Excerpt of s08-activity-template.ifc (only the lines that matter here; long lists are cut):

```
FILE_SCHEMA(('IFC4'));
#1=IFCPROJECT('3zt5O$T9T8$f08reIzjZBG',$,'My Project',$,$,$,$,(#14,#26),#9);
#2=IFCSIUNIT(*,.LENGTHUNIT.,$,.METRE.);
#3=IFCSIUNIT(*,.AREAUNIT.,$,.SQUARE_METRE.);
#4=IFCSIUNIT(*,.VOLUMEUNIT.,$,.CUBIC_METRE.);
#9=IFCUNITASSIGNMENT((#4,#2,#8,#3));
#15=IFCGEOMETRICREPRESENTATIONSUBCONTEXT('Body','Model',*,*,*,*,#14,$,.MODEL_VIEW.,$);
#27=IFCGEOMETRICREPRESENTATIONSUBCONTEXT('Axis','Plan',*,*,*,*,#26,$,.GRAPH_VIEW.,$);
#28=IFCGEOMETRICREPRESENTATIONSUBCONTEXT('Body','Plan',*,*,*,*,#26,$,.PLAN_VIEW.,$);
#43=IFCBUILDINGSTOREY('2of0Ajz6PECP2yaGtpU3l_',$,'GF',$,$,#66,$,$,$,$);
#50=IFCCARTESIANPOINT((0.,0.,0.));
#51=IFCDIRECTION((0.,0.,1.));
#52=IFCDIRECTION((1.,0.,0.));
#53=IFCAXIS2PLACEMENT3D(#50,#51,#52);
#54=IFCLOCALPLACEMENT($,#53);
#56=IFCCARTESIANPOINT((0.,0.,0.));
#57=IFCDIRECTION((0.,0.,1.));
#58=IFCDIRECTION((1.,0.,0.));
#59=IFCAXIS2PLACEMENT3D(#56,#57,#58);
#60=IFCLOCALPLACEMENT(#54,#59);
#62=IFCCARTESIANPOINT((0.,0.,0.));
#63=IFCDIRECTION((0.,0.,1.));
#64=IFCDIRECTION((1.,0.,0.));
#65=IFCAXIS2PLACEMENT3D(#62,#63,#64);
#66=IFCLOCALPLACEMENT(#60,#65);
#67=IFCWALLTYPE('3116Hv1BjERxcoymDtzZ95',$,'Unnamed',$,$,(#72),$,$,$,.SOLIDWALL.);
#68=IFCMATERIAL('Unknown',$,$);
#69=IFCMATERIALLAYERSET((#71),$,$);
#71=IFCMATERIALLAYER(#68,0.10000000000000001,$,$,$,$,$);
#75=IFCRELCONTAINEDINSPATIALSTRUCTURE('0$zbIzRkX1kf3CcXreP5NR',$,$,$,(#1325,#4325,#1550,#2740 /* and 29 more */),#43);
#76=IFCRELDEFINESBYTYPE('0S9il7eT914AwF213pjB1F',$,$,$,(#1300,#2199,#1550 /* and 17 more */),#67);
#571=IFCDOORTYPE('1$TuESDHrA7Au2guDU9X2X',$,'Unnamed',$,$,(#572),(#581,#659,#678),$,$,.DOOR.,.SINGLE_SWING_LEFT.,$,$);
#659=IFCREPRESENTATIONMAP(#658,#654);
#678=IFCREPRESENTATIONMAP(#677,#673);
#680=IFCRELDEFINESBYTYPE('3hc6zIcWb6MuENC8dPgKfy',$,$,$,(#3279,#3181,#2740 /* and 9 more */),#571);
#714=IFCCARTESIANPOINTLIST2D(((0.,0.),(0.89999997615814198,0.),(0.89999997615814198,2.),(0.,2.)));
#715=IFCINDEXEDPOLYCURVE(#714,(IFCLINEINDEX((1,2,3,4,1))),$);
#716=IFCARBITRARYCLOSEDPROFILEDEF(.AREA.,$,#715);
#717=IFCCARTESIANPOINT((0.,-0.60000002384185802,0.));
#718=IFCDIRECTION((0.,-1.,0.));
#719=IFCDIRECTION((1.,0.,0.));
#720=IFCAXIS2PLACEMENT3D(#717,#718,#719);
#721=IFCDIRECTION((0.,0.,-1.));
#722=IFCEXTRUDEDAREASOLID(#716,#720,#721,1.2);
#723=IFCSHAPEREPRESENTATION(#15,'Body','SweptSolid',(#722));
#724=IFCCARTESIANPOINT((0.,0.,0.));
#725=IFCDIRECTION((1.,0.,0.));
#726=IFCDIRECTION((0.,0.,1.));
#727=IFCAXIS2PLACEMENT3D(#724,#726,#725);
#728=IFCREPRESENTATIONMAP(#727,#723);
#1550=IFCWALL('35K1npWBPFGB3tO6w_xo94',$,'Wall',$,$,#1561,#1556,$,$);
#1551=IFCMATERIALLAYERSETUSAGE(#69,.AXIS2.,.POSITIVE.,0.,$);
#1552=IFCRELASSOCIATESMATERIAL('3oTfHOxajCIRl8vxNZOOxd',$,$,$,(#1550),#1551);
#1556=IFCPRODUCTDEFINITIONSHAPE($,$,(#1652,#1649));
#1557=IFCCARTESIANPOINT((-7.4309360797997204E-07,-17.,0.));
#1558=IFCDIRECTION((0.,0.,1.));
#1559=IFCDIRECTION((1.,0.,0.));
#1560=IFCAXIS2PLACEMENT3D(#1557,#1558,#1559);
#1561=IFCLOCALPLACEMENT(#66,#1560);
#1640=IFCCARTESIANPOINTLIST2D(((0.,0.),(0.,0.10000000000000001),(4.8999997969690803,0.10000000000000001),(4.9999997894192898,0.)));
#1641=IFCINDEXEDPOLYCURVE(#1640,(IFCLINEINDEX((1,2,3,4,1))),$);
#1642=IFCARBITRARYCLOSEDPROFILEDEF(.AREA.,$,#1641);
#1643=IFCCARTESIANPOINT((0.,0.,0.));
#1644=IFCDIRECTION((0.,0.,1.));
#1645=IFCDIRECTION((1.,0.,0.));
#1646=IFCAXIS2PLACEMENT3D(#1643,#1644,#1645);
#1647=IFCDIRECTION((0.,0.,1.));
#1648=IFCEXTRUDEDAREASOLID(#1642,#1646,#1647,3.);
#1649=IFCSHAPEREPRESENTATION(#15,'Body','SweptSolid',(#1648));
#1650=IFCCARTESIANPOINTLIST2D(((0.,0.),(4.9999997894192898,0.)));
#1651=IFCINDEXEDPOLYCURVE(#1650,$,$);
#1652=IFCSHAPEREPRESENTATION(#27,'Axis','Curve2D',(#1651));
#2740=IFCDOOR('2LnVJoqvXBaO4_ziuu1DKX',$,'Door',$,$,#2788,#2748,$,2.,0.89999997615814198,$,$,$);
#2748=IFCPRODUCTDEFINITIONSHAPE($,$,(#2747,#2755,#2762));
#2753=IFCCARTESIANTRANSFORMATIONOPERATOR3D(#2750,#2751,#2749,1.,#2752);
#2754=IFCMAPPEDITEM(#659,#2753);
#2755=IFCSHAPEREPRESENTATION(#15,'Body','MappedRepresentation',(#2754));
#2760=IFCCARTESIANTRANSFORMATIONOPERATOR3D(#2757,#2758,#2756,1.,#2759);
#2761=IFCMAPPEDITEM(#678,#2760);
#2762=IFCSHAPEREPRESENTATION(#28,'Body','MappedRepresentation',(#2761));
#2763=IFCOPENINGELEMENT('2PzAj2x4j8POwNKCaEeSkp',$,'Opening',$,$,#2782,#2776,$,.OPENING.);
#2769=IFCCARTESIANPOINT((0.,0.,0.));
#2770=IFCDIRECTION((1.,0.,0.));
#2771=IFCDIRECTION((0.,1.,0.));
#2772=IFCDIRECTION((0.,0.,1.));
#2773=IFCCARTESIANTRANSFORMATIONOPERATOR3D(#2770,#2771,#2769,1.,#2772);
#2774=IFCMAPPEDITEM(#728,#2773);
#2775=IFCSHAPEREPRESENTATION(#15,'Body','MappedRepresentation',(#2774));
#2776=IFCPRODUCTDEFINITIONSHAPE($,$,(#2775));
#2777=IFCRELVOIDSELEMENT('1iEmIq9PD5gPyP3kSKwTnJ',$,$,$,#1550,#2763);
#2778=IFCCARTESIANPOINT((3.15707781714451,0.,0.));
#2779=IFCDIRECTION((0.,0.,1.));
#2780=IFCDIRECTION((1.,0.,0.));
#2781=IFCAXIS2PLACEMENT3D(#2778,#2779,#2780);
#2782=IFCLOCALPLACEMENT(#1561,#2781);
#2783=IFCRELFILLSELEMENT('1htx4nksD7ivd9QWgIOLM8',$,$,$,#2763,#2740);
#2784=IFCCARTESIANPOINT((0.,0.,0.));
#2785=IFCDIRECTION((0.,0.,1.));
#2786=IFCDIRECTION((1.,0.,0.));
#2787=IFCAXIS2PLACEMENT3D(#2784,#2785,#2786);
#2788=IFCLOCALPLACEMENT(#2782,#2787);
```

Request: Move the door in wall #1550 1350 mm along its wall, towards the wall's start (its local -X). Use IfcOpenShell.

```python
import ifcopenshell
import ifcopenshell.api.geometry
import ifcopenshell.util.placement
import ifcopenshell.util.unit

model = ifcopenshell.open("s08-activity-template.ifc")
unit_scale = ifcopenshell.util.unit.calculate_unit_scale(model)

door = model.by_guid("2LnVJoqvXBaO4_ziuu1DKX")
opening = door.FillsVoids[0].RelatingOpeningElement
wall = opening.VoidsElements[0].RelatingBuildingElement

wall_matrix = ifcopenshell.util.placement.get_local_placement(wall.ObjectPlacement)
shift = wall_matrix[:3, 0] * -1.35 / unit_scale
before = ifcopenshell.util.placement.get_local_placement(door.ObjectPlacement)[:3, 3].copy()

# The door is placed relative to its opening, so it follows when the opening moves.
matrix = ifcopenshell.util.placement.get_local_placement(opening.ObjectPlacement)
matrix[:3, 3] += shift
ifcopenshell.api.geometry.edit_object_placement(
    model, product=opening, matrix=matrix, is_si=False, should_transform_children=True
)

after = ifcopenshell.util.placement.get_local_placement(door.ObjectPlacement)[:3, 3]
print("door moved by", (after - before).round(3) + 0.0)

model.write("s08-activity-template_rev.ifc")
```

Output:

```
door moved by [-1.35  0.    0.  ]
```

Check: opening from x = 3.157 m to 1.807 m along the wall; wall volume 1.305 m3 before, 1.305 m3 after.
